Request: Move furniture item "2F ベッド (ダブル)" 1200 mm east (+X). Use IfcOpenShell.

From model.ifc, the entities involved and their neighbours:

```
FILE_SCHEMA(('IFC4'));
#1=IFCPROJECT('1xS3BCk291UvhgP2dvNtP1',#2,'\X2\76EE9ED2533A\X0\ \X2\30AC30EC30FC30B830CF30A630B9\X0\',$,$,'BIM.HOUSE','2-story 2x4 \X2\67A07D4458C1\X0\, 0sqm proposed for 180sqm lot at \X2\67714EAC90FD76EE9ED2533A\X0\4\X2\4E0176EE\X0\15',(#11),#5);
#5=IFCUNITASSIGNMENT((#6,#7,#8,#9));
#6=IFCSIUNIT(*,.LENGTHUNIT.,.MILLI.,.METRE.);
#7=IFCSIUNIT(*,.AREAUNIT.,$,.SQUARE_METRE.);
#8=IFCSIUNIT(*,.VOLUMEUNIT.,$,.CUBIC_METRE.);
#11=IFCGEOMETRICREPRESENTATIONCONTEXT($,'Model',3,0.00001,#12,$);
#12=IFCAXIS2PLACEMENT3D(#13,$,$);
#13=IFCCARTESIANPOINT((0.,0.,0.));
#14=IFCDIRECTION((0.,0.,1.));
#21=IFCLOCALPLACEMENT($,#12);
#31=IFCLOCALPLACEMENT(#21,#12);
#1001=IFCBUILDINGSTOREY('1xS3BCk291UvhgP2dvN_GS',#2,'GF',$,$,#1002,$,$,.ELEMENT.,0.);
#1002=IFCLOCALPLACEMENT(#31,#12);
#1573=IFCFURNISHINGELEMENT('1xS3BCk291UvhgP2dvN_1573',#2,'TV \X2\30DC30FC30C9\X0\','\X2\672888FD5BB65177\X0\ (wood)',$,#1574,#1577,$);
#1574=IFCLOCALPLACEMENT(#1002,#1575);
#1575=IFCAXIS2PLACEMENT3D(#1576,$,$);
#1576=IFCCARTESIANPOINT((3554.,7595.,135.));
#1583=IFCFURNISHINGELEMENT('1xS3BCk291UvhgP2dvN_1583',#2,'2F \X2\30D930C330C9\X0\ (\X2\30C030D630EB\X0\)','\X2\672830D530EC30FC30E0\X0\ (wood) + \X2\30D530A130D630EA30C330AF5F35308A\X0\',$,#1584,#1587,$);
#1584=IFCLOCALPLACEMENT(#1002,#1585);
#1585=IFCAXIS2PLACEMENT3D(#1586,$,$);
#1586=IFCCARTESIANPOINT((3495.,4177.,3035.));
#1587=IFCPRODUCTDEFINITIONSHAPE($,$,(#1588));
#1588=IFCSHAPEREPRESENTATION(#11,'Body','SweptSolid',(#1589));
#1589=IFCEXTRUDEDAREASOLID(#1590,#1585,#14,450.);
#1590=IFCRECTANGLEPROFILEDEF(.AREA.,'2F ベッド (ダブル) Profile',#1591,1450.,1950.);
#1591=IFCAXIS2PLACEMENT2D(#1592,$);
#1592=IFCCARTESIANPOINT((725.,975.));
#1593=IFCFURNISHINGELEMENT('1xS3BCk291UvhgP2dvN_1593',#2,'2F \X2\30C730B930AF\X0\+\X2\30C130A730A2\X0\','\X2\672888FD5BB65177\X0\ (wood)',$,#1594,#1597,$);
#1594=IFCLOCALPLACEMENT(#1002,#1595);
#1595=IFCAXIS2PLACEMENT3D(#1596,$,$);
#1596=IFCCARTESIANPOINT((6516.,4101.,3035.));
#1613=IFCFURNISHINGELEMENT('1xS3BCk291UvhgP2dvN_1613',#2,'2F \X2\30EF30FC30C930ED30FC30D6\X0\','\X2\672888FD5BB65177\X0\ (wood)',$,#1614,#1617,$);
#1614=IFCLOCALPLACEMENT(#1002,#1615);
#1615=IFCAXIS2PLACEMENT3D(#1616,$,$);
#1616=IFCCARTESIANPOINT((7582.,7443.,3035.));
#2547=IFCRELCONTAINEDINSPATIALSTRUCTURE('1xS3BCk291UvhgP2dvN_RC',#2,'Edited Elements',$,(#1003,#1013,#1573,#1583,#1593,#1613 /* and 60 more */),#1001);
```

```python
import ifcopenshell
import ifcopenshell.api.geometry
import ifcopenshell.util.placement
import ifcopenshell.util.unit

model = ifcopenshell.open("model.ifc")
unit_scale = ifcopenshell.util.unit.calculate_unit_scale(model)

item = model.by_guid("1xS3BCk291UvhgP2dvN_1583")
matrix = ifcopenshell.util.placement.get_local_placement(item.ObjectPlacement)
matrix[0, 3] += 1.2 / unit_scale
ifcopenshell.api.geometry.edit_object_placement(model, product=item, matrix=matrix, is_si=False)

print(ifcopenshell.util.placement.get_local_placement(item.ObjectPlacement).round(3) + 0.0)

model.write("model-out.ifc")
```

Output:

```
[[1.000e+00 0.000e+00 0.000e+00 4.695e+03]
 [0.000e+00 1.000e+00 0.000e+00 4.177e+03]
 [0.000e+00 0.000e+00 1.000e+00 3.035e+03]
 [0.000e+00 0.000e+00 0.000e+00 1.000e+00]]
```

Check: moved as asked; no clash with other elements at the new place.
